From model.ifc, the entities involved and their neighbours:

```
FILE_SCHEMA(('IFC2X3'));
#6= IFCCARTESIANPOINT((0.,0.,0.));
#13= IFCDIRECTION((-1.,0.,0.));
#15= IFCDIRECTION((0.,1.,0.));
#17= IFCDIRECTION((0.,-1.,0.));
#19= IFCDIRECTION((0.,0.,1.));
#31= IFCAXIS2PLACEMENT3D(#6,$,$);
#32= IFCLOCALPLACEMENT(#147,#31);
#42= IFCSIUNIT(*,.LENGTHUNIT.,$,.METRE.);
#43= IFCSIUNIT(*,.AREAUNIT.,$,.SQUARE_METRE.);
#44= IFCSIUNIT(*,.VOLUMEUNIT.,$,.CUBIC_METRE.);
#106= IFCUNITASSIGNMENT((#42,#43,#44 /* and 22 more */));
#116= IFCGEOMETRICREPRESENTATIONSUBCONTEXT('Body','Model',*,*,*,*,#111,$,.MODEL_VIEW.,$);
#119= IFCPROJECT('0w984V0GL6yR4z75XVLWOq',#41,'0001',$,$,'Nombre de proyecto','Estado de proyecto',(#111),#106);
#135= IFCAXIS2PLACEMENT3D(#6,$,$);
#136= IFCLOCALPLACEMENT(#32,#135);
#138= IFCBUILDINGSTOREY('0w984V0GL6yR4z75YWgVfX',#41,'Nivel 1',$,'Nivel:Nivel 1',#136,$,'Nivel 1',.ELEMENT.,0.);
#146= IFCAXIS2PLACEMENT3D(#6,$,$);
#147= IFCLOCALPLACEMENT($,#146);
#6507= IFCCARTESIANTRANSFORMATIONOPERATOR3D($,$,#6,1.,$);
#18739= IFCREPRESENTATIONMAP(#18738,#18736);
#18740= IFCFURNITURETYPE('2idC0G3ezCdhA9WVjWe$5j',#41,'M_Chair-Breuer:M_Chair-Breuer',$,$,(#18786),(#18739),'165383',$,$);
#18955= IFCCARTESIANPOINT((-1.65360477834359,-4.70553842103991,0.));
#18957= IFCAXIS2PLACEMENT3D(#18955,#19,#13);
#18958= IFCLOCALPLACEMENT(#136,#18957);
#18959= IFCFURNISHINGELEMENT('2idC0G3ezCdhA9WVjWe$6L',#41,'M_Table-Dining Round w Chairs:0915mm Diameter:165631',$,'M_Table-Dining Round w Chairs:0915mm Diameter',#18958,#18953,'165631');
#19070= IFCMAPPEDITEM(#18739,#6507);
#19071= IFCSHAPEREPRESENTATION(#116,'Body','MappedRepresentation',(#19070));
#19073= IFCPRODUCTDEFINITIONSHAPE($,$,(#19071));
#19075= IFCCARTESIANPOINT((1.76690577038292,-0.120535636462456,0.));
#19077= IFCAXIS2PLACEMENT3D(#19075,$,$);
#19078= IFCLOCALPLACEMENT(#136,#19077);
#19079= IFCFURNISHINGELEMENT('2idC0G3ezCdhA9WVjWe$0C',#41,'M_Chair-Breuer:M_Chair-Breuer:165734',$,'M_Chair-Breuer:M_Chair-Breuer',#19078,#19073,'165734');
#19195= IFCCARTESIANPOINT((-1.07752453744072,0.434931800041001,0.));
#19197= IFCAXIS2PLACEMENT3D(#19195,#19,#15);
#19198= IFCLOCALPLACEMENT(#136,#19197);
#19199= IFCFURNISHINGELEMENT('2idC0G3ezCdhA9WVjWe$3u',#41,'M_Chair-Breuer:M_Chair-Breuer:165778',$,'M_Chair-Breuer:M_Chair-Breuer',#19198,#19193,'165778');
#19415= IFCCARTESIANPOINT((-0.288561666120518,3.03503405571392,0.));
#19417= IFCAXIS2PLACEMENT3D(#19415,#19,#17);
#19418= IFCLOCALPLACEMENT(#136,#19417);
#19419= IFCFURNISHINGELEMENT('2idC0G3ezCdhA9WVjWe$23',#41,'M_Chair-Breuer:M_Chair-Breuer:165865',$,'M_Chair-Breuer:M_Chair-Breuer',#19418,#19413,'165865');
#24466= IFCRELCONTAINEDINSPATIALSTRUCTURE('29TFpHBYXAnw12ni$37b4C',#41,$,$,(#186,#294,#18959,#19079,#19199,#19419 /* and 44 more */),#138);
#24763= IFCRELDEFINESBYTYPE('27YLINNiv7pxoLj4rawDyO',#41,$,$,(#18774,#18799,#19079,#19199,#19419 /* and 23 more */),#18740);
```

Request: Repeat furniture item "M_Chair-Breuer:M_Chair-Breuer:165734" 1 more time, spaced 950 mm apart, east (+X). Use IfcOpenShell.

```python
import numpy as np
import ifcopenshell
import ifcopenshell.api.geometry
import ifcopenshell.api.root
import ifcopenshell.util.element
import ifcopenshell.util.placement
import ifcopenshell.util.unit

model = ifcopenshell.open("model.ifc")
unit_scale = ifcopenshell.util.unit.calculate_unit_scale(model)


def reuse_history(source, copy):
    """copy_class also copies each property set's owner history, people and application; keep the originals."""
    for rel in copy.IsDefinedBy:
        if rel.is_a("IfcRelDefinesByProperties") and (history := rel.RelatingPropertyDefinition.OwnerHistory):
            rel.RelatingPropertyDefinition.OwnerHistory = source.OwnerHistory
            ifcopenshell.util.element.remove_deep2(model, history)


source = model.by_id(19079)
base = ifcopenshell.util.placement.get_local_placement(source.ObjectPlacement)
step = np.array([1.0, 0.0, 0.0]) * 0.95 / unit_scale

for i in range(1, 2):
    copy = ifcopenshell.api.root.copy_class(model, product=source)
    copy.Representation = ifcopenshell.util.element.copy_deep(
        model, source.Representation, exclude=["IfcGeometricRepresentationContext", "IfcRepresentationMap"]
    )
    copy.Name = "M_Chair-Breuer:M_Chair-Breuer"
    copy.Tag = None
    reuse_history(source, copy)
    matrix = base.copy()
    matrix[:3, 3] += i * step
    print("added at", matrix[:3, 3].round(3) + 0.0)
    ifcopenshell.api.geometry.edit_object_placement(model, product=copy, matrix=matrix, is_si=False)

model.write("model_rev.ifc")
```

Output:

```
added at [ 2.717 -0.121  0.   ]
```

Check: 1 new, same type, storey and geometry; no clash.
